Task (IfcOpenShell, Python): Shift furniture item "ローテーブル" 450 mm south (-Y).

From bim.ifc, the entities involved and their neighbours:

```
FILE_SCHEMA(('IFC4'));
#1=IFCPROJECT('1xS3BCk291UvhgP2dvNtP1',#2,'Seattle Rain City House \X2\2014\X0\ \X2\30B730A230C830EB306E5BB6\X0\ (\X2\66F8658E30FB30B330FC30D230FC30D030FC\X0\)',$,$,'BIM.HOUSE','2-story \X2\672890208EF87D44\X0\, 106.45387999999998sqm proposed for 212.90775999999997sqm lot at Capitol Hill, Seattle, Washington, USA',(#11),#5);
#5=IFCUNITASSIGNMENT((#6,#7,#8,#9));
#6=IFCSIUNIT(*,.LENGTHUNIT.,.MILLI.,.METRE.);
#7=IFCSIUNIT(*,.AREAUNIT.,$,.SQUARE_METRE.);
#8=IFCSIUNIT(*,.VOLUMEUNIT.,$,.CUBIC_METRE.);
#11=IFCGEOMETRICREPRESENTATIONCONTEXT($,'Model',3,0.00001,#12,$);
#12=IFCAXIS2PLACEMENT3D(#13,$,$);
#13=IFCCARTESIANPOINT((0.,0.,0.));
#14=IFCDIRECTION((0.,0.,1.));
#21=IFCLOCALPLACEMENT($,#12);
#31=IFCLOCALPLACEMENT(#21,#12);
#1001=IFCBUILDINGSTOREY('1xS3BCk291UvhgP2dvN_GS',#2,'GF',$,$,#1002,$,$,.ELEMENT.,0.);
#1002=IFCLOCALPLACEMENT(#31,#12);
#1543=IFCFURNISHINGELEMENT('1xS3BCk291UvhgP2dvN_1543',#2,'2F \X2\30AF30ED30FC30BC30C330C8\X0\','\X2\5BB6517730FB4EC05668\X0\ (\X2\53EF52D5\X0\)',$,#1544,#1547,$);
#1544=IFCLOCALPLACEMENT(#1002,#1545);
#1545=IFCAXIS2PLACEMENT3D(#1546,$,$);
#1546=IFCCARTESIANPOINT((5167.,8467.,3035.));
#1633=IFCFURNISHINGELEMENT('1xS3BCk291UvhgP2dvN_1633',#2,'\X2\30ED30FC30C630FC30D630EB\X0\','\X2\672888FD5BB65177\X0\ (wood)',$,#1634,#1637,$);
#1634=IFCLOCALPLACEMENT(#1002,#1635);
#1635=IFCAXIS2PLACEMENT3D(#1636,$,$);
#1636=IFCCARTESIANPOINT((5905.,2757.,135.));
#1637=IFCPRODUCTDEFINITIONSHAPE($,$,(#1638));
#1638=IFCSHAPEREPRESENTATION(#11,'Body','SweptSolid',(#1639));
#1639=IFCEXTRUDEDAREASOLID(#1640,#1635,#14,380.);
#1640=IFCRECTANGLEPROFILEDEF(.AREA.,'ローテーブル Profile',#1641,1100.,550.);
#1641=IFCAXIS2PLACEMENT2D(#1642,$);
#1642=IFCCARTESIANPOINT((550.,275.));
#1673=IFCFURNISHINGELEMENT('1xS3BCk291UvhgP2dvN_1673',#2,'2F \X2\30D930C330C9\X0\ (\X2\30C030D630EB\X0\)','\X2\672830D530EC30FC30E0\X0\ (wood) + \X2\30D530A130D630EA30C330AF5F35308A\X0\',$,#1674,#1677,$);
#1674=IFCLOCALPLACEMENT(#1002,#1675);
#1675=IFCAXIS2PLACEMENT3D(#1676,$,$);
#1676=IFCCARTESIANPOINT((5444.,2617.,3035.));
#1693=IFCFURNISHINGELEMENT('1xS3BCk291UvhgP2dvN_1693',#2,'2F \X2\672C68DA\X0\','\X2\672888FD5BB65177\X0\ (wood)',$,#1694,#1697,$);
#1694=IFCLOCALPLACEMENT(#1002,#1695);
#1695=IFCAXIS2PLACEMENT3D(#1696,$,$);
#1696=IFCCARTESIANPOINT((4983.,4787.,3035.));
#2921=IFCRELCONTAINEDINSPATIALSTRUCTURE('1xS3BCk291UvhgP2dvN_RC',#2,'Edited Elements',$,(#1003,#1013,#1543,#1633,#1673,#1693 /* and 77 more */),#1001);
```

```python
import ifcopenshell
import ifcopenshell.api.geometry
import ifcopenshell.util.placement
import ifcopenshell.util.unit

model = ifcopenshell.open("bim.ifc")
unit_scale = ifcopenshell.util.unit.calculate_unit_scale(model)

item = model.by_id(1633)
matrix = ifcopenshell.util.placement.get_local_placement(item.ObjectPlacement)
matrix[1, 3] -= 0.45 / unit_scale
ifcopenshell.api.geometry.edit_object_placement(model, product=item, matrix=matrix, is_si=False)

print(ifcopenshell.util.placement.get_local_placement(item.ObjectPlacement).round(3) + 0.0)

model.write("bim_updated.ifc")
```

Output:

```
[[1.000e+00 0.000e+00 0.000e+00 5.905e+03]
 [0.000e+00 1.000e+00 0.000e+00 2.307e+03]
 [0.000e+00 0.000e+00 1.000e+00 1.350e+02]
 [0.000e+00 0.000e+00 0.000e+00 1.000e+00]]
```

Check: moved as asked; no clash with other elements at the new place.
